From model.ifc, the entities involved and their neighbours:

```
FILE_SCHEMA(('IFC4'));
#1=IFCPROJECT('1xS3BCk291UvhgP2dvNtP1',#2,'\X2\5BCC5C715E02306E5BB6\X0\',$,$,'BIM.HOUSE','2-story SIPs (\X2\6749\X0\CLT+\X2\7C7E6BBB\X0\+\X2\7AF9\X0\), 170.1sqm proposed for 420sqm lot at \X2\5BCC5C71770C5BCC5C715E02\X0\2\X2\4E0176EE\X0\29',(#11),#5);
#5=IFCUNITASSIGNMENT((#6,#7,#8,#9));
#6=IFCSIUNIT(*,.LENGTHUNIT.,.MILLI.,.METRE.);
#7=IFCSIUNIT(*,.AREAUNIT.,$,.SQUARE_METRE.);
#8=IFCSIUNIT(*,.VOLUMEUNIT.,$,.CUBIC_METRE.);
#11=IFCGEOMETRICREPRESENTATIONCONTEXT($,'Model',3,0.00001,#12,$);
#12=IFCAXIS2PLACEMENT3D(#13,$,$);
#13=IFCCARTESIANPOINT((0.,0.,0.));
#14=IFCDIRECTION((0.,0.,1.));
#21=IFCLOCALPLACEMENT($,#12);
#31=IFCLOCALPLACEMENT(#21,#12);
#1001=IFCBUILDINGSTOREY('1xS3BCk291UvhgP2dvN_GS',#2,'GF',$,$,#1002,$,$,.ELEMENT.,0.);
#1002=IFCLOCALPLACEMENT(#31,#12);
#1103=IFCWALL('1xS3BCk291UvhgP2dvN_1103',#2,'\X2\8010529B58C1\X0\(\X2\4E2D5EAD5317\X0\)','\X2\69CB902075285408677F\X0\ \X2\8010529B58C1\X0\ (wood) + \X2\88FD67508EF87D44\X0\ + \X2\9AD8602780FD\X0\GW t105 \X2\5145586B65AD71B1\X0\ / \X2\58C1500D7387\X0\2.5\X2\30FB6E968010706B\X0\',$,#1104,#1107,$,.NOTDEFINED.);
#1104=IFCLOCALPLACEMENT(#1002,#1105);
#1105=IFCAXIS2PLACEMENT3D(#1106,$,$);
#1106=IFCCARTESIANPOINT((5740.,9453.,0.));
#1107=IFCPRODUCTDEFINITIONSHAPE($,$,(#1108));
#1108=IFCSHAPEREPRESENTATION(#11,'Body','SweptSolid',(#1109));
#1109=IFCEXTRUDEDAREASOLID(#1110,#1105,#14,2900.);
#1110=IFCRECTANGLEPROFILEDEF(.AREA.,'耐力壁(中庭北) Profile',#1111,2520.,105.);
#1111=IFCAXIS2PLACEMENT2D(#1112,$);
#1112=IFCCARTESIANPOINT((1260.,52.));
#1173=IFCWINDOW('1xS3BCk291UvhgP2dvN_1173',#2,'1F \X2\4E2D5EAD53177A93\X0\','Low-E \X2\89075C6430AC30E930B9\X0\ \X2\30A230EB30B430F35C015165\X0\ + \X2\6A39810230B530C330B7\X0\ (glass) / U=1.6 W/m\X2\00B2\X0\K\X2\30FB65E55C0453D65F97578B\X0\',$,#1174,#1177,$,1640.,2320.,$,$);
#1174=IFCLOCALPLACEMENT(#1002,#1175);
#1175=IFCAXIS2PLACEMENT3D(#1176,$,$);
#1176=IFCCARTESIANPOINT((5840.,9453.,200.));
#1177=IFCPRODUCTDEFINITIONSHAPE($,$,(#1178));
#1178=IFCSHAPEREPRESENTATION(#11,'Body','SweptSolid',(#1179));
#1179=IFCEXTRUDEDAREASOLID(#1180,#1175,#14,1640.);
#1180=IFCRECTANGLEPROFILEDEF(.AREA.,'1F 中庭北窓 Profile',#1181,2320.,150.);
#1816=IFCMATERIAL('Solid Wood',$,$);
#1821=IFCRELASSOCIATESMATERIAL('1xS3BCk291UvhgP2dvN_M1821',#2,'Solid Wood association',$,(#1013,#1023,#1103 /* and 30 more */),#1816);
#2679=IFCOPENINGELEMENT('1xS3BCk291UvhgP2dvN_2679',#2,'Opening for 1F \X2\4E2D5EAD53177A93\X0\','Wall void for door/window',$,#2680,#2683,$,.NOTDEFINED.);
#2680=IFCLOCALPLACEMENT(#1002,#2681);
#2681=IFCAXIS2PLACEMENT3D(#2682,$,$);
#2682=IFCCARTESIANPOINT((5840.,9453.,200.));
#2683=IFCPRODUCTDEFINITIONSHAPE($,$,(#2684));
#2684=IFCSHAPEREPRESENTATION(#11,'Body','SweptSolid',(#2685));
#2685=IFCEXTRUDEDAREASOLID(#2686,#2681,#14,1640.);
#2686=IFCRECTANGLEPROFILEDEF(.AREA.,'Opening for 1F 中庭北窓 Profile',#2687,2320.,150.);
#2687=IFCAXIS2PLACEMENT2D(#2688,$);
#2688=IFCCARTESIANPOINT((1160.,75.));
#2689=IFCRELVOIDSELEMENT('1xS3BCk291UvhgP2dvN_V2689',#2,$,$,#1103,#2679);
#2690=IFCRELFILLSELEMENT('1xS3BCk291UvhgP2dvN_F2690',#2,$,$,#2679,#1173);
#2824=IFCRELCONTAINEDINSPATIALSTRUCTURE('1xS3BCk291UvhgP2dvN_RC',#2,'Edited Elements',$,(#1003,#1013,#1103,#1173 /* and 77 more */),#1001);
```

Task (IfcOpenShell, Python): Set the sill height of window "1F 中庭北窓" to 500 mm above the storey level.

```python
import numpy as np
import ifcopenshell
import ifcopenshell.api.geometry
import ifcopenshell.geom
import ifcopenshell.util.element
import ifcopenshell.util.placement
import ifcopenshell.util.shape
import ifcopenshell.util.unit

model = ifcopenshell.open("model.ifc")
unit_scale = ifcopenshell.util.unit.calculate_unit_scale(model)

window = model.by_id(1173)
opening = window.FillsVoids[0].RelatingOpeningElement
storey = ifcopenshell.util.element.get_container(window, ifc_class="IfcBuildingStorey")
level = ifcopenshell.util.placement.get_local_placement(storey.ObjectPlacement)[2, 3]

# The opening's origin need not be at the sill, so measure its lowest point.
shape = ifcopenshell.geom.create_shape(ifcopenshell.geom.settings(), opening)
bottom = ifcopenshell.util.shape.get_shape_bottom_elevation(shape, shape.geometry) / unit_scale
dz = level + 500.0 - bottom

shift = np.array([0.0, 0.0, dz])
# The window is not placed relative to its opening, so move both.
for product in (opening, window):
    matrix = ifcopenshell.util.placement.get_local_placement(product.ObjectPlacement)
    matrix[:3, 3] += shift
    ifcopenshell.api.geometry.edit_object_placement(model, product=product, matrix=matrix, is_si=False)

print(f"moved by {dz * unit_scale:+.3f} m")

model.write("model_rev.ifc")
```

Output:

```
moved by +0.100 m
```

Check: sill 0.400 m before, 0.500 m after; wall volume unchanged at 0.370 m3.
